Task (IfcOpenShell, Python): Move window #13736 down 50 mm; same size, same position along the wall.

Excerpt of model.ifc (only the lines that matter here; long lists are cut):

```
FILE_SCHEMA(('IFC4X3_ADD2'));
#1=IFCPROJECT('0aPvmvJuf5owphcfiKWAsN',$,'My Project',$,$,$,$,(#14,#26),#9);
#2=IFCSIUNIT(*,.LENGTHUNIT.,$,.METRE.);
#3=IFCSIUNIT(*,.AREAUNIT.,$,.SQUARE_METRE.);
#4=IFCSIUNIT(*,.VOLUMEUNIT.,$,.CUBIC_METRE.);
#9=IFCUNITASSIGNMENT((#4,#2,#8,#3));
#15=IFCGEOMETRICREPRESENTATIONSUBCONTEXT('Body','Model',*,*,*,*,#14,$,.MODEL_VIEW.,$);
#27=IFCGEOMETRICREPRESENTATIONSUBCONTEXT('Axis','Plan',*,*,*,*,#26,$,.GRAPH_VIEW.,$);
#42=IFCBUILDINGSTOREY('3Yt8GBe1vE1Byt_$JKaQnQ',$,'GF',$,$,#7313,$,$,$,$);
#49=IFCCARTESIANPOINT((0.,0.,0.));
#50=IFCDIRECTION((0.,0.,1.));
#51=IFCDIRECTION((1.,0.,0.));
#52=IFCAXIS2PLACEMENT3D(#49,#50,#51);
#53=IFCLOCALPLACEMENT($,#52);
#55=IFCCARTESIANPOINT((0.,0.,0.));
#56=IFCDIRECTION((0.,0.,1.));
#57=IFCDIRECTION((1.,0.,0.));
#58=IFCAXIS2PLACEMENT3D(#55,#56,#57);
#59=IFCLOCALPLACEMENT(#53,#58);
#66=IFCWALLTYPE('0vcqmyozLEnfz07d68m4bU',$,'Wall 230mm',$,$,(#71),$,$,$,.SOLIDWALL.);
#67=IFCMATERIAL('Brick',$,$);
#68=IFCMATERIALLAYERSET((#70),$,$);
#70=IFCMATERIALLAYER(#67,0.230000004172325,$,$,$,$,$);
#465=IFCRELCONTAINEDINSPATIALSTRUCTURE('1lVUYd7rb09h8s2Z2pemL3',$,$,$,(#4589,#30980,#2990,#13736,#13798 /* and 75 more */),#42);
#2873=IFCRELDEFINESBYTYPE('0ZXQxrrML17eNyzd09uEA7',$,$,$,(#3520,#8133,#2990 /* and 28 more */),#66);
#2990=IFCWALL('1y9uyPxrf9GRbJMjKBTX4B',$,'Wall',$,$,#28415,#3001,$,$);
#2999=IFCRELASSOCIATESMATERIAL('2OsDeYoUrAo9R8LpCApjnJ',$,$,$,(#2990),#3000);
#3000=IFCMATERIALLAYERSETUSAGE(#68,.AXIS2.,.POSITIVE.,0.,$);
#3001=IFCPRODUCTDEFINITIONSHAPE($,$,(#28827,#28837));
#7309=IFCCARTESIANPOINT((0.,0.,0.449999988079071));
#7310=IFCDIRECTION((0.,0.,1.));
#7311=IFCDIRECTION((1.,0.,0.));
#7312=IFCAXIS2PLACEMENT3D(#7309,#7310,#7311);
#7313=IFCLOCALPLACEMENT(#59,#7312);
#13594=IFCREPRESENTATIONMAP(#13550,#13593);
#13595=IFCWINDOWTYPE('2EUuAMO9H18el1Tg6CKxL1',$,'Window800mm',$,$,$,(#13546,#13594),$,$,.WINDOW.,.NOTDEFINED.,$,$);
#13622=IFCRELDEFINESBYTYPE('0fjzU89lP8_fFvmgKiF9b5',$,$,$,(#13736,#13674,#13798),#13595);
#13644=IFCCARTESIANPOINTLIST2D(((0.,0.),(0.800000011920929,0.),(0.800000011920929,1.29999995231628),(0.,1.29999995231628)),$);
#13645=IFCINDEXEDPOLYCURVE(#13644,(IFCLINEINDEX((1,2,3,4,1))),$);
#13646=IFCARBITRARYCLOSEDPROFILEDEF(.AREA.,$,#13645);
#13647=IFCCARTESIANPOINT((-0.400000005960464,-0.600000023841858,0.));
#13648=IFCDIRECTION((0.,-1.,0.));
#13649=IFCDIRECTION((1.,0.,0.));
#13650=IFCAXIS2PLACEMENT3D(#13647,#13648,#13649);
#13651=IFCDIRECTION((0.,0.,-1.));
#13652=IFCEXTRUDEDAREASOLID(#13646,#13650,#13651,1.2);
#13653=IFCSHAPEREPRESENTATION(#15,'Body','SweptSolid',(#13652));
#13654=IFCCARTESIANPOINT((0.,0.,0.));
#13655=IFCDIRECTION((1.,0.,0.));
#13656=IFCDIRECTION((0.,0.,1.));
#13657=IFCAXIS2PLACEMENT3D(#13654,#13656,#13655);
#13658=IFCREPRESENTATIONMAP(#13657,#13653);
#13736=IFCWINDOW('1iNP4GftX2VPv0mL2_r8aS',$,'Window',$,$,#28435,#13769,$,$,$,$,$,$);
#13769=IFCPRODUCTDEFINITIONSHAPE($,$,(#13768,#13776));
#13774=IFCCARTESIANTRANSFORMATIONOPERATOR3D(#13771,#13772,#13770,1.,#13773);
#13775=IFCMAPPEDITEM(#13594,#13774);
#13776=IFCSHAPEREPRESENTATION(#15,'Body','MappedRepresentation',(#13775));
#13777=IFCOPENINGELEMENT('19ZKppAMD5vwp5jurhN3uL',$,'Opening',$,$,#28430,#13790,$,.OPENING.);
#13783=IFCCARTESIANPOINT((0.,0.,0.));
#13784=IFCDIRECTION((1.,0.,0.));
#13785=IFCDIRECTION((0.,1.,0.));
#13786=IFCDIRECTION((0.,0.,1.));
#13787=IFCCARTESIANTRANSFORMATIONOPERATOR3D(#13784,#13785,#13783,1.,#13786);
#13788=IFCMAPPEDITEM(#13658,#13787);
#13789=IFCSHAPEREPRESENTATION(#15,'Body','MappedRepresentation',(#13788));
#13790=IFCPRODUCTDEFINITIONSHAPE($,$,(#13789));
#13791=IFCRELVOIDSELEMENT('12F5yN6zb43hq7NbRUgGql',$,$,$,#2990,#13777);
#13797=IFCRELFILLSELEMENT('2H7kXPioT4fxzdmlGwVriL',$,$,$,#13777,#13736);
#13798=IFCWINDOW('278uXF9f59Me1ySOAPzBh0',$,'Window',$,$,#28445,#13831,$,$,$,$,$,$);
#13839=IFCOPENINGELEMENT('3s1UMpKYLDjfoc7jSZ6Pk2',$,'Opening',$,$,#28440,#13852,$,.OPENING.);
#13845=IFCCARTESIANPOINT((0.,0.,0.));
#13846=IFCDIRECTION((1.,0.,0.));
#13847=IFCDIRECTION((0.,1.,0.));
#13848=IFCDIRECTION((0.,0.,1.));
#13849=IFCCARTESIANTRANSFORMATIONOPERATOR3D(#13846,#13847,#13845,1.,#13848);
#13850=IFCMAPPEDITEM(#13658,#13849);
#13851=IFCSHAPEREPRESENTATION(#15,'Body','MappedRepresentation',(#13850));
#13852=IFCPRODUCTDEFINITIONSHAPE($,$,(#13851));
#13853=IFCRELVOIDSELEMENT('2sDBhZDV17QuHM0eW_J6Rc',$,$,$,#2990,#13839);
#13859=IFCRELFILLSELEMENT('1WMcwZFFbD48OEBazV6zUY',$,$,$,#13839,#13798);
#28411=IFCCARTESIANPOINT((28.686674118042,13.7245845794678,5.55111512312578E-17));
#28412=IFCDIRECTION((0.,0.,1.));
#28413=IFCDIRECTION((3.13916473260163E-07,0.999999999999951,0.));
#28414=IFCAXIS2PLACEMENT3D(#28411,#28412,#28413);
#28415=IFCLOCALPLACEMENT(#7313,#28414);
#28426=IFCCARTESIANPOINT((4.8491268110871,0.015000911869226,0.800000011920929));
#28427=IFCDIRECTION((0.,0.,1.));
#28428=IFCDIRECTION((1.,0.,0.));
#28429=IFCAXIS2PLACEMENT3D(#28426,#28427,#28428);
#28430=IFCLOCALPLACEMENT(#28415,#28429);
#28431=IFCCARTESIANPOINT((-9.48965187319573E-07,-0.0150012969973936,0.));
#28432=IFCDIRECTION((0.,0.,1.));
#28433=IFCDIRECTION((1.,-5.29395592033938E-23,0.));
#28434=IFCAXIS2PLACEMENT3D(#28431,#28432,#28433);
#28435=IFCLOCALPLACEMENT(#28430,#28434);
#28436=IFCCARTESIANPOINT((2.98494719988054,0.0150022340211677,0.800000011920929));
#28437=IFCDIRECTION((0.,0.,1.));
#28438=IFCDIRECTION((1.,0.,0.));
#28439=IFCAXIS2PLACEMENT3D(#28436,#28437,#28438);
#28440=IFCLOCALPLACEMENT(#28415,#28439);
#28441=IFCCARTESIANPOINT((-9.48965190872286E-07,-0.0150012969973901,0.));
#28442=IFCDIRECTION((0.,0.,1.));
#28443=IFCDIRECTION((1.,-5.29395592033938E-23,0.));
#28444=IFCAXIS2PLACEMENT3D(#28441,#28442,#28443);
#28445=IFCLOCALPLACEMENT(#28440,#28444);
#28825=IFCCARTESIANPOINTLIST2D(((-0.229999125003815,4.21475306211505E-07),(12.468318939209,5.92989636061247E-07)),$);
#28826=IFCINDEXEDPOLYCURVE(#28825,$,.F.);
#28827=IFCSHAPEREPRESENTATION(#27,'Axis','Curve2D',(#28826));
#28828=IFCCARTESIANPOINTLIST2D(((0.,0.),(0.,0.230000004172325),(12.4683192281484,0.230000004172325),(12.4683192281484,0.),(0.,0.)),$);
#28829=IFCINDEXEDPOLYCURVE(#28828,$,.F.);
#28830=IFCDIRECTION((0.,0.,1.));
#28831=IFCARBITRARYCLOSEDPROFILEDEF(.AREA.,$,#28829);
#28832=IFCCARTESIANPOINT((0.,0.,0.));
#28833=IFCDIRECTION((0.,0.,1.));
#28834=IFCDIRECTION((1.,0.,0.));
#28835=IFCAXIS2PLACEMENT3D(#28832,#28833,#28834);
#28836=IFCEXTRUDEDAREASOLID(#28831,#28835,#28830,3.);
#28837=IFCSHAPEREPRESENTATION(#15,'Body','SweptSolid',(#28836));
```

```python
import numpy as np
import ifcopenshell
import ifcopenshell.api.geometry
import ifcopenshell.util.placement
import ifcopenshell.util.unit

model = ifcopenshell.open("model.ifc")
unit_scale = ifcopenshell.util.unit.calculate_unit_scale(model)

window = model.by_guid("1iNP4GftX2VPv0mL2_r8aS")
opening = window.FillsVoids[0].RelatingOpeningElement
dz = -0.05

shift = np.array([0.0, 0.0, dz])
# The window is placed relative to its opening, so it follows when the opening moves.
matrix = ifcopenshell.util.placement.get_local_placement(opening.ObjectPlacement)
matrix[:3, 3] += shift
ifcopenshell.api.geometry.edit_object_placement(
    model, product=opening, matrix=matrix, is_si=False, should_transform_children=True
)

print(f"moved by {dz * unit_scale:+.3f} m")

model.write("model_v2.ifc")
```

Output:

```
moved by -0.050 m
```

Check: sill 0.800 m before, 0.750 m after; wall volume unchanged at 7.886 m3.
